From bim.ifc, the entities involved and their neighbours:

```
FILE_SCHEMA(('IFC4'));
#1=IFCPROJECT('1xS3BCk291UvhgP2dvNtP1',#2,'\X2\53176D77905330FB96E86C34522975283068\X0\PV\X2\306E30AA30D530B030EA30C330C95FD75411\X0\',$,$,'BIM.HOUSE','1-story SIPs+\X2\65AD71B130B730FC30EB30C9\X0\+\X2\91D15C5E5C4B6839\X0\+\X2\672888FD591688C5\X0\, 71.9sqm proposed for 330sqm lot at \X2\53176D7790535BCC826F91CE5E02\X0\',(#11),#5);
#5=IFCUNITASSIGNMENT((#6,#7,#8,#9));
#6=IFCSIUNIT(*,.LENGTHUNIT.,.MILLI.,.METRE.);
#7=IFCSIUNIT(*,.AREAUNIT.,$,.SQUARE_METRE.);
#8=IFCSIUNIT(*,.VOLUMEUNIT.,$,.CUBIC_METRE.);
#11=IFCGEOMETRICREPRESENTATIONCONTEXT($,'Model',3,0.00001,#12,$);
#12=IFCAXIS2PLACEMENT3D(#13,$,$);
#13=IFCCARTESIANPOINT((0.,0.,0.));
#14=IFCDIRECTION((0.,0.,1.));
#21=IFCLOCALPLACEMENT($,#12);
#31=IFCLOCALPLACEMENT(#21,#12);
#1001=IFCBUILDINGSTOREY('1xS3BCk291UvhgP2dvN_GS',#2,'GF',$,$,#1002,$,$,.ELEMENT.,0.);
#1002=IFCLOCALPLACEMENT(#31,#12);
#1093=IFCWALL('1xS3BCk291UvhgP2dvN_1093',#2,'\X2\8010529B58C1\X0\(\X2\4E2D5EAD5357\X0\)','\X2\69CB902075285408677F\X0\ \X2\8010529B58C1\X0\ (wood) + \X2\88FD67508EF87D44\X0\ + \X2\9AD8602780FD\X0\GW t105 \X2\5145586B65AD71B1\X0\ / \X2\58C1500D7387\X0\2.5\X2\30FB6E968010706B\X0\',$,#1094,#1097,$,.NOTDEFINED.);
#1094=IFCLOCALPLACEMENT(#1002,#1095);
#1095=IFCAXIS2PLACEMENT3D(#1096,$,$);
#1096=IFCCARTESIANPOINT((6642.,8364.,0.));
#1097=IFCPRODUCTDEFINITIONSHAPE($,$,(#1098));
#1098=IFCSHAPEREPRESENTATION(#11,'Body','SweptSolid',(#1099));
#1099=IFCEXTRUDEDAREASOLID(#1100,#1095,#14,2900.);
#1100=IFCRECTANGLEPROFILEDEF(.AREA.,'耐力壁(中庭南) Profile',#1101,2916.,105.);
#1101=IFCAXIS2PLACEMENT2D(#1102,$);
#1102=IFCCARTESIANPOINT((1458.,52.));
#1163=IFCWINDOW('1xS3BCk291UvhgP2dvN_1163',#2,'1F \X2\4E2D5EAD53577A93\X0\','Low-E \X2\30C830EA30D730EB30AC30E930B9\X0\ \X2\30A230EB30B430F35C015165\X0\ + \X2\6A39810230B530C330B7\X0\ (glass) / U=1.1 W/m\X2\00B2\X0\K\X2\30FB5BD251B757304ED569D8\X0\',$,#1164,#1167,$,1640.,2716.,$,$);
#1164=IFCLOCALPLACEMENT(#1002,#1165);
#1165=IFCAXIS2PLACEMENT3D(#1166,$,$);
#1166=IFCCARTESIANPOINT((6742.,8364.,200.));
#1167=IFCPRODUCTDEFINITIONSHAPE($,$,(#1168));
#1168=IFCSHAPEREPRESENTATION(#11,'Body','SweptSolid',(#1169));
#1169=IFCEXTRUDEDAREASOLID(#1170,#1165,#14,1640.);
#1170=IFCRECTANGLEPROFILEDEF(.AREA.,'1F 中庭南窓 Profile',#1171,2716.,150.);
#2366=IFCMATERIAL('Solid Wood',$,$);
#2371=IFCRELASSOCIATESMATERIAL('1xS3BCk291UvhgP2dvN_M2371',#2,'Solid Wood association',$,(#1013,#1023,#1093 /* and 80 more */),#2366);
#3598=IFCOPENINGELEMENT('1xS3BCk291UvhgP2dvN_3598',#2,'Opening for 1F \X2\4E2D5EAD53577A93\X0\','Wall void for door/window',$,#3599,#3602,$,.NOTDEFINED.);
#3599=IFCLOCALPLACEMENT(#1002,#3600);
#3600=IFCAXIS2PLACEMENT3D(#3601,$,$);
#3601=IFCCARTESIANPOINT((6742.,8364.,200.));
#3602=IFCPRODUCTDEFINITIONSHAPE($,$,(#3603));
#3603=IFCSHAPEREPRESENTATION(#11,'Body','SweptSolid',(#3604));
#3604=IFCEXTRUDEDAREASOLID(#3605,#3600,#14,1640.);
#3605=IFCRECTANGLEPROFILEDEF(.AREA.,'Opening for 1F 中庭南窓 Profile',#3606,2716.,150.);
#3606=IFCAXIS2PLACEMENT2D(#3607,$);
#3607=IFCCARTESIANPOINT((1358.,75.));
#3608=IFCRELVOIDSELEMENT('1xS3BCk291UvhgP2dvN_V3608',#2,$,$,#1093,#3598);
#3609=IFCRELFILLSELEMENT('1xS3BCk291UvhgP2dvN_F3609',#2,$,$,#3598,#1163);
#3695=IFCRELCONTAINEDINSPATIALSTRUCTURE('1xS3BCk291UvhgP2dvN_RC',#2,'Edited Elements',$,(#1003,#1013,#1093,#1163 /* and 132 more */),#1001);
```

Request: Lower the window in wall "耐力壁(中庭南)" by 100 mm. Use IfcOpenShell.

```python
import numpy as np
import ifcopenshell
import ifcopenshell.api.geometry
import ifcopenshell.util.placement
import ifcopenshell.util.unit

model = ifcopenshell.open("bim.ifc")
unit_scale = ifcopenshell.util.unit.calculate_unit_scale(model)

window = model.by_guid("1xS3BCk291UvhgP2dvN_1163")
opening = window.FillsVoids[0].RelatingOpeningElement
dz = -0.1 / unit_scale

shift = np.array([0.0, 0.0, dz])
# The window is not placed relative to its opening, so move both.
for product in (opening, window):
    matrix = ifcopenshell.util.placement.get_local_placement(product.ObjectPlacement)
    matrix[:3, 3] += shift
    ifcopenshell.api.geometry.edit_object_placement(model, product=product, matrix=matrix, is_si=False)

print(f"moved by {dz * unit_scale:+.3f} m")

model.write("bim_v2.ifc")
```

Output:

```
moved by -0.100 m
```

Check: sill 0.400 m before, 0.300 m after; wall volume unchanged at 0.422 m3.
